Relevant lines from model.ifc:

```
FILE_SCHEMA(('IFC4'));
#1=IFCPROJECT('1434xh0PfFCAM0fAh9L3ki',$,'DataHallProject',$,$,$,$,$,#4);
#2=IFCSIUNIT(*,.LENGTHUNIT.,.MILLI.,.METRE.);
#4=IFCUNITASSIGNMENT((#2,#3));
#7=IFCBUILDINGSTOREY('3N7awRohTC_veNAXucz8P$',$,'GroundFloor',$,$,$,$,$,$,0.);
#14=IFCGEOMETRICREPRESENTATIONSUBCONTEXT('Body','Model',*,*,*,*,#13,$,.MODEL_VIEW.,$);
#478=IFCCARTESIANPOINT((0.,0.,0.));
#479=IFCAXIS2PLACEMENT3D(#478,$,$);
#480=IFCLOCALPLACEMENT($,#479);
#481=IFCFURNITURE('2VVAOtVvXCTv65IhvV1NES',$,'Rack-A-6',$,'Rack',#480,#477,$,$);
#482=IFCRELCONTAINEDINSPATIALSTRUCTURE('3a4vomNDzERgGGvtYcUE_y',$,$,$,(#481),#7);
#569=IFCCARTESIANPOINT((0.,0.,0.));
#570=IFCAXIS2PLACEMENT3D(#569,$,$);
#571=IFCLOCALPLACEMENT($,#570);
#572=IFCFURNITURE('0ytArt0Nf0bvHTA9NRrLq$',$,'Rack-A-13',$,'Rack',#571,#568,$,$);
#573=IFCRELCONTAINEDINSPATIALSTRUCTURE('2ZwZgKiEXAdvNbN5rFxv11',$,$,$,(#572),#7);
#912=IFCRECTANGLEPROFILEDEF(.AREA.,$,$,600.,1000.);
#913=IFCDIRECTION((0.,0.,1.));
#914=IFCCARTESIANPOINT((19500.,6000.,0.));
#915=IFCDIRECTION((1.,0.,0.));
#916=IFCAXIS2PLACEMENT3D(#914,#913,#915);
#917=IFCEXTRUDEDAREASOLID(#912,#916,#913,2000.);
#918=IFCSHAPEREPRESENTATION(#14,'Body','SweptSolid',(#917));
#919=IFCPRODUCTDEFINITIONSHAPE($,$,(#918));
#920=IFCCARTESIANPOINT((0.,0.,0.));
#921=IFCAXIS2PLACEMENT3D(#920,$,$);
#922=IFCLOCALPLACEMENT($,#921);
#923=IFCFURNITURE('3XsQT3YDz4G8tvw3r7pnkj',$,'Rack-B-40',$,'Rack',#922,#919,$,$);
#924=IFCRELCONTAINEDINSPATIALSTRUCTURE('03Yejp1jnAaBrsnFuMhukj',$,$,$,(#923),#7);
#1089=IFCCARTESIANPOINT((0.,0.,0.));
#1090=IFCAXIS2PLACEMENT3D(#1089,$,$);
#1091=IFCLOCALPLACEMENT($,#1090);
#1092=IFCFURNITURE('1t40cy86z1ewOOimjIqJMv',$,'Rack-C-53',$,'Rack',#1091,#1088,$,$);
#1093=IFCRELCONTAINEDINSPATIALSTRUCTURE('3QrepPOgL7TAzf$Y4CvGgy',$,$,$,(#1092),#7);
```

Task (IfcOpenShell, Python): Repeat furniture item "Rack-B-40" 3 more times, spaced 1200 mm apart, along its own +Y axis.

```python
import ifcopenshell
import ifcopenshell.api.geometry
import ifcopenshell.api.root
import ifcopenshell.util.element
import ifcopenshell.util.placement
import ifcopenshell.util.unit

model = ifcopenshell.open("model.ifc")
unit_scale = ifcopenshell.util.unit.calculate_unit_scale(model)

source = model.by_guid("3XsQT3YDz4G8tvw3r7pnkj")
base = ifcopenshell.util.placement.get_local_placement(source.ObjectPlacement)
step = base[:3, 1] * 1.2 / unit_scale

for i in range(1, 4):
    copy = ifcopenshell.api.root.copy_class(model, product=source)
    copy.Representation = ifcopenshell.util.element.copy_deep(
        model, source.Representation, exclude=["IfcGeometricRepresentationContext", "IfcRepresentationMap"]
    )
    matrix = base.copy()
    matrix[:3, 3] += i * step
    print("added at", matrix[:3, 3].round(3) + 0.0)
    ifcopenshell.api.geometry.edit_object_placement(model, product=copy, matrix=matrix, is_si=False)

model.write("model_v2.ifc")
```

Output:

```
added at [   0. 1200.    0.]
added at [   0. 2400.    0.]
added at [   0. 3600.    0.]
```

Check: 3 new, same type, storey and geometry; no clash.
